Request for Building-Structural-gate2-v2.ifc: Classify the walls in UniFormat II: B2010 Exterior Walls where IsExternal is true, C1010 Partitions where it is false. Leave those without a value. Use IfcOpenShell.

First a look at what the model holds.

```python
import ifcopenshell
import ifcopenshell.util.element

model = ifcopenshell.open("Building-Structural-gate2-v2.ifc")
print(model.schema)
print("classifications:", [c.Name for c in model.by_type("IfcClassification")])
values = [ifcopenshell.util.element.get_pset(e, "Pset_WallCommon", "IsExternal") for e in model.by_type("IfcWall")]
for value in (True, False, None):
    print("IsExternal", value, values.count(value))
```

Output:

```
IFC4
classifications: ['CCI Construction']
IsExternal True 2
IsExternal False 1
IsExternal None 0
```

```python
import ifcopenshell
import ifcopenshell.api.classification
import ifcopenshell.util.element

model = ifcopenshell.open("Building-Structural-gate2-v2.ifc")

system = ifcopenshell.api.classification.add_classification(model, classification="UniFormat II")

walls = model.by_type("IfcWall")
external = {e: ifcopenshell.util.element.get_pset(e, "Pset_WallCommon", "IsExternal") for e in walls}
for flag, code, name in ((True, "B2010", "Exterior Walls"), (False, "C1010", "Partitions")):
    products = [e for e in walls if external[e] is flag]
    ifcopenshell.api.classification.add_reference(
        model, products=products, classification=system, identification=code, name=name
    )
    print(code, len(products))

model.write("Building-Structural-gate2-v2_updated.ifc")
```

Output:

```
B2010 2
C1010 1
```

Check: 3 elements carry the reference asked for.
